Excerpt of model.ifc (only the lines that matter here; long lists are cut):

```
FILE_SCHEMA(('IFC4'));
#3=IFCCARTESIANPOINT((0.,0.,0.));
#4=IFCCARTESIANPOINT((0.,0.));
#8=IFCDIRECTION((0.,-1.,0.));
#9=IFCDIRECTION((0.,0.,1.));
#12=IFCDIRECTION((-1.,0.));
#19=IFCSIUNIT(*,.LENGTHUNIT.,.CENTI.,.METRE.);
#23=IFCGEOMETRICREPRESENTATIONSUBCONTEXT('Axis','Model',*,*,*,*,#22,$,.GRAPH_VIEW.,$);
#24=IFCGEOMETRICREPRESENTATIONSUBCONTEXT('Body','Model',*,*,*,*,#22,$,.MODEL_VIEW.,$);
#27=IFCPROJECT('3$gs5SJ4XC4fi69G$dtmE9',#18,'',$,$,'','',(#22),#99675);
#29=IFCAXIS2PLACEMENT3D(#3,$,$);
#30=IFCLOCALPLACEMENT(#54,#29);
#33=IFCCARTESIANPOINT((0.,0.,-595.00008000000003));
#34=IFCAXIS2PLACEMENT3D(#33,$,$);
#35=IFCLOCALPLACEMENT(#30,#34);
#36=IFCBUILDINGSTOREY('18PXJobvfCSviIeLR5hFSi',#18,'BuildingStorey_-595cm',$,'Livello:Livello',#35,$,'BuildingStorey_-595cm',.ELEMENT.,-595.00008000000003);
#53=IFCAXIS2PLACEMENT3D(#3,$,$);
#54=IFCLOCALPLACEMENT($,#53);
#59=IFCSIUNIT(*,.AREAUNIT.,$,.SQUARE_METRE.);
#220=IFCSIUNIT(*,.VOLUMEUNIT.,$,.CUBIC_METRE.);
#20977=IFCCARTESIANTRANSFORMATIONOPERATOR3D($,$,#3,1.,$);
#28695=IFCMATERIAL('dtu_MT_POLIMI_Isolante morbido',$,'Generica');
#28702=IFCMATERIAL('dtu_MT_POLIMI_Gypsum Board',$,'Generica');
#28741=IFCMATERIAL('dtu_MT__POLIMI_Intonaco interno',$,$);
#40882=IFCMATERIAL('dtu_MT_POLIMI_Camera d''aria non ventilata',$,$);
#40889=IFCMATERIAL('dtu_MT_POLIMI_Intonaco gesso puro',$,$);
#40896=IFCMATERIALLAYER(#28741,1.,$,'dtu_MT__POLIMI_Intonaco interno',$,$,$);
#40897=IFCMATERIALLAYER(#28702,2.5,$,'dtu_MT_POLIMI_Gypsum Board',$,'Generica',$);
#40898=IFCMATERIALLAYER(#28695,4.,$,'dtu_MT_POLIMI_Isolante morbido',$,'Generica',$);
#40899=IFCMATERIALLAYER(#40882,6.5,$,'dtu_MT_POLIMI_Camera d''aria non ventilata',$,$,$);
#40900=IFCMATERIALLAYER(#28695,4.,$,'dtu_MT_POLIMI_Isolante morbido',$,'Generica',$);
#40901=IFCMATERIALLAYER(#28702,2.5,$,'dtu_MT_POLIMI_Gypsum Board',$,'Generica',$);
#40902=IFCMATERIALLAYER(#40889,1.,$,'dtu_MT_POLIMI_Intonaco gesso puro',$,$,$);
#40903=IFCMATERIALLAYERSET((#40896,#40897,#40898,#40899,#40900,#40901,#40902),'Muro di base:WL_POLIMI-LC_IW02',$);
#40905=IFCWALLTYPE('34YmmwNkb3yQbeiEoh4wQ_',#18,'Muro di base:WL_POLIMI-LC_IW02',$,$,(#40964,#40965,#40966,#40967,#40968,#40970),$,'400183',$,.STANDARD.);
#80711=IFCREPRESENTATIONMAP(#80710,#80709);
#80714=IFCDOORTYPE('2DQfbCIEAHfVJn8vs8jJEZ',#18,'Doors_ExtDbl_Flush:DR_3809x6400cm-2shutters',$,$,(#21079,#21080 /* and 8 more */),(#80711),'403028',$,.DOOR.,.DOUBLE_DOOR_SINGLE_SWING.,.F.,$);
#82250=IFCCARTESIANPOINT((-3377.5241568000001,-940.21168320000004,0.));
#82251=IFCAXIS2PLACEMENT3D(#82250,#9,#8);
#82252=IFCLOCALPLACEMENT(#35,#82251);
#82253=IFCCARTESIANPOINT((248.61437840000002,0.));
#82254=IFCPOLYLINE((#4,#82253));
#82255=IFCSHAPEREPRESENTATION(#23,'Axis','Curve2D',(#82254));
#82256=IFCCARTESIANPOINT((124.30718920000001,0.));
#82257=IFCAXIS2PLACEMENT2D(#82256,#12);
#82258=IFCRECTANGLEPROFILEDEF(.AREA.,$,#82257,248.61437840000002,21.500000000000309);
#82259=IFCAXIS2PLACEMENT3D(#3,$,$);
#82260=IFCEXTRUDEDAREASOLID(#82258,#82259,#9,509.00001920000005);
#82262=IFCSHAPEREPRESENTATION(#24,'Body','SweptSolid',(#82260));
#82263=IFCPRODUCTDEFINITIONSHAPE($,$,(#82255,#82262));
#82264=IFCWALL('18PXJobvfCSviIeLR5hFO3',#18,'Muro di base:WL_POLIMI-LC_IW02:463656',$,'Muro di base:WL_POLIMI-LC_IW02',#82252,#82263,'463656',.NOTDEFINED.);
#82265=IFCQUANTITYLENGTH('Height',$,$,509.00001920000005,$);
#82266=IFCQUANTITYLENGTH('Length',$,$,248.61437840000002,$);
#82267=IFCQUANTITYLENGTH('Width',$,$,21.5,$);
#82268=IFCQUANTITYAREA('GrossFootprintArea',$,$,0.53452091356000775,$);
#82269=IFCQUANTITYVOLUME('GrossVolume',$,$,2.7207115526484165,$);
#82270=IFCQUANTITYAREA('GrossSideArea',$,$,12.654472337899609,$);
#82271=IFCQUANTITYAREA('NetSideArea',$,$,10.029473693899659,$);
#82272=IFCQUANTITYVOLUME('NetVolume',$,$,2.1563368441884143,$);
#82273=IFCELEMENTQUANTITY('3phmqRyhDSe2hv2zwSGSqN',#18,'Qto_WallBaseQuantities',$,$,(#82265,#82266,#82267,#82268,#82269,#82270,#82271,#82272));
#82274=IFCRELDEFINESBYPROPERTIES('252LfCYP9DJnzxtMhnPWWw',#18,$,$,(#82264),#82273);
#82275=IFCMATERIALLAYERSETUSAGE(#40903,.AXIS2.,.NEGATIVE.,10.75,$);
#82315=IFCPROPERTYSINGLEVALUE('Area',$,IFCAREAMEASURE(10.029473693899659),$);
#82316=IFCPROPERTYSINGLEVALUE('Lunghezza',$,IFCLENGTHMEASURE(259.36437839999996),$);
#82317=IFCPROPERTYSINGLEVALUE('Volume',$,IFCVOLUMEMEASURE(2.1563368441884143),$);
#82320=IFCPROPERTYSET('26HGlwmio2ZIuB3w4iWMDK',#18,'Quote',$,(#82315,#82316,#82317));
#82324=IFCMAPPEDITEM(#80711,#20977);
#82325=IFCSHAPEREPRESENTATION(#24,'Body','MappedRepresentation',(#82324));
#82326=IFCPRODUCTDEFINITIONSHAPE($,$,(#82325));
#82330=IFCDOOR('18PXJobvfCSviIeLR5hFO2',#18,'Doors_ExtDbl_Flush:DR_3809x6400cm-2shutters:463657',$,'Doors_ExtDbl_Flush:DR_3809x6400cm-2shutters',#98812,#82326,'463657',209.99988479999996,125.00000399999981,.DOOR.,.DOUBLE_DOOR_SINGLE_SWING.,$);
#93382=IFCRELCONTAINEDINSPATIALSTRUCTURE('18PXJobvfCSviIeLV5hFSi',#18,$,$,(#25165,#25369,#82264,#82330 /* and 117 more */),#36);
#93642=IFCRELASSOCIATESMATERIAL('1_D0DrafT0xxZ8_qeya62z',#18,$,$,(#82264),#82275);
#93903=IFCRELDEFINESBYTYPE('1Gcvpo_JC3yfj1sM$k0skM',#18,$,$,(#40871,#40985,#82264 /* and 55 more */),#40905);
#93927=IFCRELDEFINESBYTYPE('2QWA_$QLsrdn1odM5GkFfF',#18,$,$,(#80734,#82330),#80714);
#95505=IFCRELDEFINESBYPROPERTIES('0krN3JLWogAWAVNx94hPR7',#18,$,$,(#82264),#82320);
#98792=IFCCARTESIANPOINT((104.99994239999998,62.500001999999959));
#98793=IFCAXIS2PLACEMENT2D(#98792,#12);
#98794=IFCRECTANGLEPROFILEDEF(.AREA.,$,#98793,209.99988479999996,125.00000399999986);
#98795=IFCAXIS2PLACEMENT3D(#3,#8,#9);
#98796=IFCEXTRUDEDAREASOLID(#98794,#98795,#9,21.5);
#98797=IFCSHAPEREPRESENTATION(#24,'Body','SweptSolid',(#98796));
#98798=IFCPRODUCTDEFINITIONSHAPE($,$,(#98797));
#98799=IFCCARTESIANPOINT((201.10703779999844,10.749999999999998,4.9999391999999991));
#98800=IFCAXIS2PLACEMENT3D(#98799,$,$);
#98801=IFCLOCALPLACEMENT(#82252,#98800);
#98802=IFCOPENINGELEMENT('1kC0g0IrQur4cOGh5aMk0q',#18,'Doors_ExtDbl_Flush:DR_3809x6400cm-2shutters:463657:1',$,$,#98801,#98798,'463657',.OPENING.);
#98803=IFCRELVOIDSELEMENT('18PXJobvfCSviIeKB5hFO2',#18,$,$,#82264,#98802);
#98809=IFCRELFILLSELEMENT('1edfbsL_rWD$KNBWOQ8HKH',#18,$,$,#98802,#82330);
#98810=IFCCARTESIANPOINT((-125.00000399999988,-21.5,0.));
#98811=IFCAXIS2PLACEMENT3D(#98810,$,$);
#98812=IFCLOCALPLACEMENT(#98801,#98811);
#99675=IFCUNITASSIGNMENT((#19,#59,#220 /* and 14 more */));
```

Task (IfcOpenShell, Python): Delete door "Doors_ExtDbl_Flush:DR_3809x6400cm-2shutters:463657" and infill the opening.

```python
import ifcopenshell
import ifcopenshell.api.feature
import ifcopenshell.api.pset
import ifcopenshell.api.root
import ifcopenshell.geom
import ifcopenshell.util.element
import ifcopenshell.util.shape
import ifcopenshell.util.unit

model = ifcopenshell.open("model.ifc")
area_scale = ifcopenshell.util.unit.calculate_unit_scale(model, "AREAUNIT")
volume_scale = ifcopenshell.util.unit.calculate_unit_scale(model, "VOLUMEUNIT")
settings = ifcopenshell.geom.settings()


def volume(element):
    """Net volume in cubic metres, openings subtracted."""
    shape = ifcopenshell.geom.create_shape(settings, element)
    return ifcopenshell.util.shape.get_volume(shape.geometry)


door = model.by_guid("18PXJobvfCSviIeLR5hFO2")
opening = door.FillsVoids[0].RelatingOpeningElement
wall = opening.VoidsElements[0].RelatingBuildingElement
before = volume(wall)

ifcopenshell.api.root.remove_product(model, product=door)
ifcopenshell.api.feature.remove_feature(model, feature=opening)

after = volume(wall)
thickness = 0.215  # wall thickness in metres

# Update the wall's stored quantities.
qto = model.by_id(ifcopenshell.util.element.get_pset(wall, "Qto_WallBaseQuantities", should_inherit=False)["id"])
ifcopenshell.api.pset.edit_qto(model, qto=qto, properties={
    "NetSideArea": after / thickness / area_scale,
    "NetVolume": after / volume_scale,
})
pset = model.by_id(ifcopenshell.util.element.get_pset(wall, "Quote", should_inherit=False)["id"])
ifcopenshell.api.pset.edit_pset(model, pset=pset, properties={
    "Area": model.create_entity("IfcAreaMeasure", after / thickness / area_scale),
    "Volume": model.create_entity("IfcVolumeMeasure", after / volume_scale),
})

print(f"wall volume {before:.3f} -> {after:.3f} m3")

model.write("model_edited.ifc")
```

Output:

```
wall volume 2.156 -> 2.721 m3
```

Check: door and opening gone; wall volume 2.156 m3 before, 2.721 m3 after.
